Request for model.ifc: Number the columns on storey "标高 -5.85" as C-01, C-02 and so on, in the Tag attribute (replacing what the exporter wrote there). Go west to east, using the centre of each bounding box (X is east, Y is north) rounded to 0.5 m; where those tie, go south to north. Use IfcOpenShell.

First a look at what the model holds.

```python
import ifcopenshell
import ifcopenshell.util.element
import ifcopenshell.util.placement

model = ifcopenshell.open("model.ifc")
print(model.schema)
storey = next(s for s in model.by_type("IfcBuildingStorey") if s.Name == "标高 -5.85")
columns = [e for e in ifcopenshell.util.element.get_decomposition(storey) if e.is_a("IfcColumn")]
for e in sorted(columns, key=lambda e: e.id()):
    origin = ifcopenshell.util.placement.get_local_placement(e.ObjectPlacement)[:3, 3]
    print(e.id(), e.Tag, e.Name, origin.round(2) + 0.0, sep=" | ")
```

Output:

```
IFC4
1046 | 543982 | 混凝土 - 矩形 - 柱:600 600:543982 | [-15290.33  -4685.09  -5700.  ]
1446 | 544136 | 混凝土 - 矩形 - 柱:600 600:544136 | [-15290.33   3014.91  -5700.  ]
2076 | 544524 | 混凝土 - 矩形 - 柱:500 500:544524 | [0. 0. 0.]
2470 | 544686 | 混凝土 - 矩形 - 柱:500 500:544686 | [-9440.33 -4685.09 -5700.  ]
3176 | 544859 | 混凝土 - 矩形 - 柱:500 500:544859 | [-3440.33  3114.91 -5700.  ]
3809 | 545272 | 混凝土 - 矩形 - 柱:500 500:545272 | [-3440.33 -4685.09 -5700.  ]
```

```python
import ifcopenshell
import ifcopenshell.geom
import ifcopenshell.util.element
import ifcopenshell.util.shape

model = ifcopenshell.open("model.ifc")
settings = ifcopenshell.geom.settings()
settings.set("use-world-coords", True)


def centre(element):
    shape = ifcopenshell.geom.create_shape(settings, element)
    return ifcopenshell.util.shape.get_bbox_centroid(shape.geometry)


storey = next(s for s in model.by_type("IfcBuildingStorey") if s.Name == "标高 -5.85")
columns = [e for e in ifcopenshell.util.element.get_decomposition(storey) if e.is_a("IfcColumn")]

# Insertion points can sit at a corner or the storey origin, so sort by the geometry (in metres).
centres = {e: centre(e) for e in columns}
columns.sort(key=lambda e: (round(centres[e][0] / 0.5), centres[e][1]))

for i, e in enumerate(columns, start=1):
    number = f"C-{i:02d}"
    e.Tag = number
    print(e.id(), number)

model.write("model_v2.ifc")
```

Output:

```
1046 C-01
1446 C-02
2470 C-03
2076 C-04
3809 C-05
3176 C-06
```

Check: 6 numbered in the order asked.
